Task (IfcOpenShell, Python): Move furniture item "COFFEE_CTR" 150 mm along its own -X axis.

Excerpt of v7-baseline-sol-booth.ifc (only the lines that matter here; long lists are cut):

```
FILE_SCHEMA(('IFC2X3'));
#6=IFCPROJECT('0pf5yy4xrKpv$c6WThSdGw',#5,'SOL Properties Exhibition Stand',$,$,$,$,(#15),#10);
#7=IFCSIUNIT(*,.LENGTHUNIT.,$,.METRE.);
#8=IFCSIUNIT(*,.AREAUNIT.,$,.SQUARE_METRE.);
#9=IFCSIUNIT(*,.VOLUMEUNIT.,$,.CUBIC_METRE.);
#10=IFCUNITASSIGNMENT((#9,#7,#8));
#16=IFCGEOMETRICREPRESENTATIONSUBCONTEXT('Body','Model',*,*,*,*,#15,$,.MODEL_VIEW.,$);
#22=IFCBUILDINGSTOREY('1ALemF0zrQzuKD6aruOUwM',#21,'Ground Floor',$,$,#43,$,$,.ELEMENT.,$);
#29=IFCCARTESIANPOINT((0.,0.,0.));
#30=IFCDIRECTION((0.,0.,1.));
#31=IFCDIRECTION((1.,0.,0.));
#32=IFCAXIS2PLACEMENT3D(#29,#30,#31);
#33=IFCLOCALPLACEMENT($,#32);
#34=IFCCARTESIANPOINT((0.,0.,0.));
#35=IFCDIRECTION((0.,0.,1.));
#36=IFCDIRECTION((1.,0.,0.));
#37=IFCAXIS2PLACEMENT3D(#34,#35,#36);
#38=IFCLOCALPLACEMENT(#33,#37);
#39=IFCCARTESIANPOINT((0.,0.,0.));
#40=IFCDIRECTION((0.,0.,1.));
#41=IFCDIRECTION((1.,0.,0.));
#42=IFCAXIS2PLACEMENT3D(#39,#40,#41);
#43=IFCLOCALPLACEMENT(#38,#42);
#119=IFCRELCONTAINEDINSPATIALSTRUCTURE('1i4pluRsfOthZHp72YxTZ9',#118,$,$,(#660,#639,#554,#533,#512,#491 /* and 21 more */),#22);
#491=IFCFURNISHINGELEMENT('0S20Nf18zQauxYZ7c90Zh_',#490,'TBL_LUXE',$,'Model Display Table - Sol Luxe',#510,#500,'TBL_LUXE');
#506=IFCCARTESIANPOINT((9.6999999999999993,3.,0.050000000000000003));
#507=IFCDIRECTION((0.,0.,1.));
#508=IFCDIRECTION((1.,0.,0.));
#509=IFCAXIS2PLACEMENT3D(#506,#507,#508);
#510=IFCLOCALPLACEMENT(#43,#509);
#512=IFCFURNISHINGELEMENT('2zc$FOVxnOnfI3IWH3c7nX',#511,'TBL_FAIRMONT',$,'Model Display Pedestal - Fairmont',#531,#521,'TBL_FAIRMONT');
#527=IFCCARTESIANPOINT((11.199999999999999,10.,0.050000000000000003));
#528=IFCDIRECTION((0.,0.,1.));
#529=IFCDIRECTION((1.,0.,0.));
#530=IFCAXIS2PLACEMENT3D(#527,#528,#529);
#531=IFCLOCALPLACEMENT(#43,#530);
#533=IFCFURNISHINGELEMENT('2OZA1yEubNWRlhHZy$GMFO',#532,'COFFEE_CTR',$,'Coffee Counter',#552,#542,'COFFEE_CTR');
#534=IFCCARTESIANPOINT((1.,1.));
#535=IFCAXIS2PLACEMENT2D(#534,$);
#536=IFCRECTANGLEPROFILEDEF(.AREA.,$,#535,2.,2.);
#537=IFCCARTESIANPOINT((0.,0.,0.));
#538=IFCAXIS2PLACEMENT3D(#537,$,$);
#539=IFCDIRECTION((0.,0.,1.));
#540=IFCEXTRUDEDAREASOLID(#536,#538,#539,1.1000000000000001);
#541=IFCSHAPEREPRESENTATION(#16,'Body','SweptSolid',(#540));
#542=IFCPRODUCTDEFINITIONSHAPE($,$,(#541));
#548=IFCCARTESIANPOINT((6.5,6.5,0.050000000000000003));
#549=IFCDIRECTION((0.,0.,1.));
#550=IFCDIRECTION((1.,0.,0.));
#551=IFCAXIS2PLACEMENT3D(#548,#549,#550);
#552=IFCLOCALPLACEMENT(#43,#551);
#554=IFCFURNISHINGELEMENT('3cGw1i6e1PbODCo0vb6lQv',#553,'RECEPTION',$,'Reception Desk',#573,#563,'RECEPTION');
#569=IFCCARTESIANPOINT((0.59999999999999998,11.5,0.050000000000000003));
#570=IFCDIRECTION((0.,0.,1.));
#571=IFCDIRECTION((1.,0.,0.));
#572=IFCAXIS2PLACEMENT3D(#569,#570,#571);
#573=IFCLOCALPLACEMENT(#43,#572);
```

```python
import ifcopenshell
import ifcopenshell.api.geometry
import ifcopenshell.util.placement

model = ifcopenshell.open("v7-baseline-sol-booth.ifc")

item = model.by_id(533)
matrix = ifcopenshell.util.placement.get_local_placement(item.ObjectPlacement)
matrix[:3, 3] -= matrix[:3, 0] * 0.15
ifcopenshell.api.geometry.edit_object_placement(model, product=item, matrix=matrix, is_si=False)

print(ifcopenshell.util.placement.get_local_placement(item.ObjectPlacement).round(3) + 0.0)

model.write("v7-baseline-sol-booth_updated.ifc")
```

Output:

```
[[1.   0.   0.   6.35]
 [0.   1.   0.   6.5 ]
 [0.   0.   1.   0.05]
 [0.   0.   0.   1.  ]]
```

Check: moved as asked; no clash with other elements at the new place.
